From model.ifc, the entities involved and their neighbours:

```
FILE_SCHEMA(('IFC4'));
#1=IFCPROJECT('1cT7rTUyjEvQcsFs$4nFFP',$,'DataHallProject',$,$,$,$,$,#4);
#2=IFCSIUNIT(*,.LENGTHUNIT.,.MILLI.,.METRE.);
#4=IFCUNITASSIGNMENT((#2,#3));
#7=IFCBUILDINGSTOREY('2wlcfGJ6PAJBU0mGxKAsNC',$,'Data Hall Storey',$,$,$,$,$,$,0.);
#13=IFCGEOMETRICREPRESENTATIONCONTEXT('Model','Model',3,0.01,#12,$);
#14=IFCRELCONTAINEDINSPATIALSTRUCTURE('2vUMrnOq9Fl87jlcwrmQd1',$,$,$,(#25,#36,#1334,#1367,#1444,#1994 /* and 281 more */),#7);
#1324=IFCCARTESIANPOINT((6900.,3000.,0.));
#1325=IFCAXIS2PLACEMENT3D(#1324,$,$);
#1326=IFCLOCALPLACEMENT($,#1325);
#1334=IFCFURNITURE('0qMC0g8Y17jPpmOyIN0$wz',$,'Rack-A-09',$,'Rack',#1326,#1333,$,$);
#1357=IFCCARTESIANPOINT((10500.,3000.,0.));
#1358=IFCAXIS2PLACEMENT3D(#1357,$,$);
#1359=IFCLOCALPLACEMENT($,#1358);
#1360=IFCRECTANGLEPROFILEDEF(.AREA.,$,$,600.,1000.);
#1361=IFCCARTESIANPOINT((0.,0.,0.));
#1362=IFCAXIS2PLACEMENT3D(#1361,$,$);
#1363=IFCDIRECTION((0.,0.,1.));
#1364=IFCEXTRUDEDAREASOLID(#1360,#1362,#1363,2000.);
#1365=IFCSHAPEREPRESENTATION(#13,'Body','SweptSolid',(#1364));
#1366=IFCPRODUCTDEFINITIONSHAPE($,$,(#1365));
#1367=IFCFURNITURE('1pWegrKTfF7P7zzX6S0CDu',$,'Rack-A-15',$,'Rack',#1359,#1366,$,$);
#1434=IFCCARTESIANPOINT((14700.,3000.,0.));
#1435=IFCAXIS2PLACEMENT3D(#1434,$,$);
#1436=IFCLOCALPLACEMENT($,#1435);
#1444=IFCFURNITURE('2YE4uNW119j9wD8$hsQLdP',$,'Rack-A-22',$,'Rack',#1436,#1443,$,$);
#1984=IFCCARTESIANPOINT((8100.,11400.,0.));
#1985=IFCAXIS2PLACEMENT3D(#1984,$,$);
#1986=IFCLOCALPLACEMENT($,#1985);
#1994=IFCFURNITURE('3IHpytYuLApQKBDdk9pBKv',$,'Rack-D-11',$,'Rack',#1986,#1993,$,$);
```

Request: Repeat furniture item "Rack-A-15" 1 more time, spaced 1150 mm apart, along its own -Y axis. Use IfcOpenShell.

```python
import ifcopenshell
import ifcopenshell.api.geometry
import ifcopenshell.api.root
import ifcopenshell.util.element
import ifcopenshell.util.placement
import ifcopenshell.util.unit

model = ifcopenshell.open("model.ifc")
unit_scale = ifcopenshell.util.unit.calculate_unit_scale(model)

source = model.by_guid("1pWegrKTfF7P7zzX6S0CDu")
base = ifcopenshell.util.placement.get_local_placement(source.ObjectPlacement)
step = -base[:3, 1] * 1.15 / unit_scale

for i in range(1, 2):
    copy = ifcopenshell.api.root.copy_class(model, product=source)
    copy.Representation = ifcopenshell.util.element.copy_deep(
        model, source.Representation, exclude=["IfcGeometricRepresentationContext", "IfcRepresentationMap"]
    )
    matrix = base.copy()
    matrix[:3, 3] += i * step
    print("added at", matrix[:3, 3].round(3) + 0.0)
    ifcopenshell.api.geometry.edit_object_placement(model, product=copy, matrix=matrix, is_si=False)

model.write("model_v2.ifc")
```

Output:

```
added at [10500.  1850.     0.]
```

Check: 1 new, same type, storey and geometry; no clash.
